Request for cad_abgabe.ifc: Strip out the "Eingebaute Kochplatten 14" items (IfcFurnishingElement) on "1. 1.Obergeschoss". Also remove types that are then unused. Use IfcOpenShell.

First a look at what the model holds.

```python
import ifcopenshell
import ifcopenshell.util.element

model = ifcopenshell.open("cad_abgabe.ifc")
print(model.schema)
storey = next(s for s in model.by_type("IfcBuildingStorey") if s.Name == "1. 1.Obergeschoss")
furniture = [e for e in ifcopenshell.util.element.get_decomposition(storey) if e.is_a("IfcFurnishingElement")]
seen = {}
for e in furniture:
    element_type = ifcopenshell.util.element.get_type(e)
    name = element_type.Name if element_type not in (None, e) else None
    seen[name] = seen.get(name, 0) + 1
for name, count in sorted(seen.items(), key=str):
    print(count, "x", name)
```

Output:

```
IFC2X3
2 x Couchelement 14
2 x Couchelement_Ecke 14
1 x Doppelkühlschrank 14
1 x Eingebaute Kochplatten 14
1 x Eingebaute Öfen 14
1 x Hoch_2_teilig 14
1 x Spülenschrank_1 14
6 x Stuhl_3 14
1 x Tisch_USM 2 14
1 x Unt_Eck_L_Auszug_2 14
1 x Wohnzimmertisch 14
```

```python
import ifcopenshell
import ifcopenshell.api.root
import ifcopenshell.util.element

model = ifcopenshell.open("cad_abgabe.ifc")

storey = next(s for s in model.by_type("IfcBuildingStorey") if s.Name == "1. 1.Obergeschoss")
furniture = [e for e in ifcopenshell.util.element.get_decomposition(storey) if e.is_a("IfcFurnishingElement")]
targets = [e for e in furniture if (t := ifcopenshell.util.element.get_type(e)) not in (None, e) and t.Name == "Eingebaute Kochplatten 14"]
types = {ifcopenshell.util.element.get_type(e) for e in targets} - {None, *targets}

for e in targets:
    ifcopenshell.api.root.remove_product(model, product=e)
print(len(targets), "removed")

unused = [t for t in types if not ifcopenshell.util.element.get_types(t)]
for t in unused:
    ifcopenshell.api.root.remove_product(model, product=t)
print(len(unused), "unused types removed")

model.write("cad_abgabe_rev.ifc")
```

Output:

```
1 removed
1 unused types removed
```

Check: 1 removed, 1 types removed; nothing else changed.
